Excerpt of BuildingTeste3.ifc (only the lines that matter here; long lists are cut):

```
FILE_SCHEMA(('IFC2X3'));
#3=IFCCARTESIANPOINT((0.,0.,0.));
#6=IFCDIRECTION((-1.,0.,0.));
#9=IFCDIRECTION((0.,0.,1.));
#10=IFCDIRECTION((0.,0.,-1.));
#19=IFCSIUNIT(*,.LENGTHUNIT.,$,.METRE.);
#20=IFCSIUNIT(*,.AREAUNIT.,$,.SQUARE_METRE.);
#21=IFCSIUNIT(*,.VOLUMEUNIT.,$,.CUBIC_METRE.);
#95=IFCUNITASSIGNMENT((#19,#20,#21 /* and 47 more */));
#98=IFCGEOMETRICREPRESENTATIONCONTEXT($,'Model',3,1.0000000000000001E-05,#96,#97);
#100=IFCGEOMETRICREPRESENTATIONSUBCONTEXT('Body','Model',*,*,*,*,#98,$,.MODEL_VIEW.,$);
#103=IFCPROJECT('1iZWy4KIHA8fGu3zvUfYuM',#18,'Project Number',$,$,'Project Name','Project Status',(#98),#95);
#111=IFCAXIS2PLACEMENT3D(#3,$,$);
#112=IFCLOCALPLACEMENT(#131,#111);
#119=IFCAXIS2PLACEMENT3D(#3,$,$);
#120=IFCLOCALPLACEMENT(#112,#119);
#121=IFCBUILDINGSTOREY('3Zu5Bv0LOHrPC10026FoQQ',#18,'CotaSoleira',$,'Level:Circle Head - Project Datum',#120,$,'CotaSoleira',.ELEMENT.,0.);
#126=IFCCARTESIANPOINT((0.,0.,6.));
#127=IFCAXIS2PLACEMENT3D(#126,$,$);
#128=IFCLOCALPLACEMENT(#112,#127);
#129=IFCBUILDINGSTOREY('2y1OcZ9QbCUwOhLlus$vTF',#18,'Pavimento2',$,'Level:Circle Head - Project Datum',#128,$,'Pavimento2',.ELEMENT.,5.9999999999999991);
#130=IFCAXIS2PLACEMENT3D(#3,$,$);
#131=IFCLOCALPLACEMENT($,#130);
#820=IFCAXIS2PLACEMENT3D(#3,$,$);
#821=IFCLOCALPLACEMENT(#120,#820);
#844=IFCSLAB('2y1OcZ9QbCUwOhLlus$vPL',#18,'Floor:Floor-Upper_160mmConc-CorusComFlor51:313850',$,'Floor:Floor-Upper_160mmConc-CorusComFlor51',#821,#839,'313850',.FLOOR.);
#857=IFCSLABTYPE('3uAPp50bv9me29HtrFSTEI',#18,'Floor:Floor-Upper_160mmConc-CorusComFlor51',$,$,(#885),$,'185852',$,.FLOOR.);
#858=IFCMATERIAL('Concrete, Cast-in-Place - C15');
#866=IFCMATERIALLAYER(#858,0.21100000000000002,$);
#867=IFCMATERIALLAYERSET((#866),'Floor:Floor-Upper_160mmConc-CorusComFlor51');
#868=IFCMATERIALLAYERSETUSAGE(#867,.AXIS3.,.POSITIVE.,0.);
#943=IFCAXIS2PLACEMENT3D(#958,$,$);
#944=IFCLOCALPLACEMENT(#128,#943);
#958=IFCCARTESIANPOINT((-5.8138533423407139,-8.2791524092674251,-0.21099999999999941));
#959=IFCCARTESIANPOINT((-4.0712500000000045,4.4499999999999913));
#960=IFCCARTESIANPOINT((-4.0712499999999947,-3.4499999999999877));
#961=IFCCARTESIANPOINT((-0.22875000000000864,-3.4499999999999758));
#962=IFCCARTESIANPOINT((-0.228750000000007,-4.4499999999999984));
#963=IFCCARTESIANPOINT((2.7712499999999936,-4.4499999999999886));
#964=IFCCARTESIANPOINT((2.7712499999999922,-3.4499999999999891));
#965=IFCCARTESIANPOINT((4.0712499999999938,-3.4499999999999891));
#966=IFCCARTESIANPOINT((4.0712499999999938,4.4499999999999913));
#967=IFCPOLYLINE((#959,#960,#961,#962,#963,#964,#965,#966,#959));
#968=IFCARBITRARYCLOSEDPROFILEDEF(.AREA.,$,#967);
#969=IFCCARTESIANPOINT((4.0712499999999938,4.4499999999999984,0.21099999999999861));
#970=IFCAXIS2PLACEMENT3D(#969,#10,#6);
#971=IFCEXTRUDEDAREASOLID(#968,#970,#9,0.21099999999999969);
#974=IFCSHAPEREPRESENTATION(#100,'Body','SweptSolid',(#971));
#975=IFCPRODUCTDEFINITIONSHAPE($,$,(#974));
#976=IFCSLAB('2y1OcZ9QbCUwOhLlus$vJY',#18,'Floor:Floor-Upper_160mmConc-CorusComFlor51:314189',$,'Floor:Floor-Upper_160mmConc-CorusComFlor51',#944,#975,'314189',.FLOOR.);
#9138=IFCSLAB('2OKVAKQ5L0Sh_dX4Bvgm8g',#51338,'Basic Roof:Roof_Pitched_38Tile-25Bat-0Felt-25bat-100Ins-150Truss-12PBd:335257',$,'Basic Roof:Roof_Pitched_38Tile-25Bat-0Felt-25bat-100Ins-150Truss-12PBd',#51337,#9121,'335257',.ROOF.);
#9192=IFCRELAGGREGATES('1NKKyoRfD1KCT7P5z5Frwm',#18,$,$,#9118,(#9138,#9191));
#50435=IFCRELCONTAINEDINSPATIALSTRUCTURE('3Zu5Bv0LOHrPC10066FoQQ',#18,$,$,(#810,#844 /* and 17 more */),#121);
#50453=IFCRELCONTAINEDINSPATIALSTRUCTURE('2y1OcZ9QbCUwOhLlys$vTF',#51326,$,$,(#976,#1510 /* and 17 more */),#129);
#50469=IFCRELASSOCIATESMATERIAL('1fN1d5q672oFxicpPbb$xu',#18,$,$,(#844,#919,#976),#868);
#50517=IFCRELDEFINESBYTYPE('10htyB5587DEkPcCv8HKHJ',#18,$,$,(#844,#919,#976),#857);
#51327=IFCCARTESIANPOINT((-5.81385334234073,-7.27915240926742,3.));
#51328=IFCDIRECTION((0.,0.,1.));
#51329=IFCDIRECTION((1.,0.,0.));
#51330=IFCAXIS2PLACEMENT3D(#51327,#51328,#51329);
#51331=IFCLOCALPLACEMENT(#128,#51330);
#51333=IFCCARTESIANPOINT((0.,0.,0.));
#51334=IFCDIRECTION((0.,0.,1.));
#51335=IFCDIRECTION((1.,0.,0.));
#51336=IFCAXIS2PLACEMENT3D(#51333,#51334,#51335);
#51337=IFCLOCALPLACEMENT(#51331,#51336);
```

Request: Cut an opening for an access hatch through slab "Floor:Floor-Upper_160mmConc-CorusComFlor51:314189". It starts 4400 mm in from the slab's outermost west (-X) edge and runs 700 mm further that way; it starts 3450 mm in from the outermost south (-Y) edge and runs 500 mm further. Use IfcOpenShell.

```python
import numpy as np
import ifcopenshell
import ifcopenshell.api.feature
import ifcopenshell.api.geometry
import ifcopenshell.api.root
import ifcopenshell.geom
import ifcopenshell.util.placement
import ifcopenshell.util.representation
import ifcopenshell.util.shape
import ifcopenshell.util.unit

model = ifcopenshell.open("BuildingTeste3.ifc")
unit_scale = ifcopenshell.util.unit.calculate_unit_scale(model)
settings = ifcopenshell.geom.settings()


def volume(element):
    """Net volume in cubic metres, openings subtracted."""
    shape = ifcopenshell.geom.create_shape(settings, element)
    return ifcopenshell.util.shape.get_volume(shape.geometry)


slab = model.by_id(976)
before = volume(slab)

# Extent in the slab's own axes, in metres. The edges named are its -X and -Y sides.
slab_shape = ifcopenshell.geom.create_shape(settings, slab)
vertices = ifcopenshell.util.shape.get_vertices(slab_shape.geometry)
x_min, y_min, bottom = vertices.min(axis=0)
top = vertices[:, 2].max()

opening = ifcopenshell.api.root.create_entity(model, ifc_class="IfcOpeningElement", name="Access hatch opening")
context = ifcopenshell.util.representation.get_context(model, "Model", "Body", "MODEL_VIEW")
width, depth = 0.7, 0.5
outline = [(0.0, 0.0), (width, 0.0), (width, depth), (0.0, depth), (0.0, 0.0)]
# Overshoot both faces by 50 mm so the cut is clean.
shape = ifcopenshell.api.geometry.add_slab_representation(
    model, context=context, depth=top - bottom + 0.1, polyline=outline
)
ifcopenshell.api.geometry.assign_representation(model, product=opening, representation=shape)

matrix = ifcopenshell.util.placement.get_local_placement(slab.ObjectPlacement)
matrix[:, 3] = matrix @ np.append(np.array([x_min + 4.4, y_min + 3.45, bottom - 0.05]) / unit_scale, 1.0)
ifcopenshell.api.geometry.edit_object_placement(model, product=opening, matrix=matrix, is_si=False)
ifcopenshell.api.feature.add_feature(model, feature=opening, element=slab)

after = volume(slab)

print(f"slab volume {before:.3f} -> {after:.3f} m3")

model.write("BuildingTeste3_rev.ifc")
```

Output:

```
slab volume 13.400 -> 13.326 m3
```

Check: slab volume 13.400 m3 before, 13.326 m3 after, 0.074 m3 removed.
